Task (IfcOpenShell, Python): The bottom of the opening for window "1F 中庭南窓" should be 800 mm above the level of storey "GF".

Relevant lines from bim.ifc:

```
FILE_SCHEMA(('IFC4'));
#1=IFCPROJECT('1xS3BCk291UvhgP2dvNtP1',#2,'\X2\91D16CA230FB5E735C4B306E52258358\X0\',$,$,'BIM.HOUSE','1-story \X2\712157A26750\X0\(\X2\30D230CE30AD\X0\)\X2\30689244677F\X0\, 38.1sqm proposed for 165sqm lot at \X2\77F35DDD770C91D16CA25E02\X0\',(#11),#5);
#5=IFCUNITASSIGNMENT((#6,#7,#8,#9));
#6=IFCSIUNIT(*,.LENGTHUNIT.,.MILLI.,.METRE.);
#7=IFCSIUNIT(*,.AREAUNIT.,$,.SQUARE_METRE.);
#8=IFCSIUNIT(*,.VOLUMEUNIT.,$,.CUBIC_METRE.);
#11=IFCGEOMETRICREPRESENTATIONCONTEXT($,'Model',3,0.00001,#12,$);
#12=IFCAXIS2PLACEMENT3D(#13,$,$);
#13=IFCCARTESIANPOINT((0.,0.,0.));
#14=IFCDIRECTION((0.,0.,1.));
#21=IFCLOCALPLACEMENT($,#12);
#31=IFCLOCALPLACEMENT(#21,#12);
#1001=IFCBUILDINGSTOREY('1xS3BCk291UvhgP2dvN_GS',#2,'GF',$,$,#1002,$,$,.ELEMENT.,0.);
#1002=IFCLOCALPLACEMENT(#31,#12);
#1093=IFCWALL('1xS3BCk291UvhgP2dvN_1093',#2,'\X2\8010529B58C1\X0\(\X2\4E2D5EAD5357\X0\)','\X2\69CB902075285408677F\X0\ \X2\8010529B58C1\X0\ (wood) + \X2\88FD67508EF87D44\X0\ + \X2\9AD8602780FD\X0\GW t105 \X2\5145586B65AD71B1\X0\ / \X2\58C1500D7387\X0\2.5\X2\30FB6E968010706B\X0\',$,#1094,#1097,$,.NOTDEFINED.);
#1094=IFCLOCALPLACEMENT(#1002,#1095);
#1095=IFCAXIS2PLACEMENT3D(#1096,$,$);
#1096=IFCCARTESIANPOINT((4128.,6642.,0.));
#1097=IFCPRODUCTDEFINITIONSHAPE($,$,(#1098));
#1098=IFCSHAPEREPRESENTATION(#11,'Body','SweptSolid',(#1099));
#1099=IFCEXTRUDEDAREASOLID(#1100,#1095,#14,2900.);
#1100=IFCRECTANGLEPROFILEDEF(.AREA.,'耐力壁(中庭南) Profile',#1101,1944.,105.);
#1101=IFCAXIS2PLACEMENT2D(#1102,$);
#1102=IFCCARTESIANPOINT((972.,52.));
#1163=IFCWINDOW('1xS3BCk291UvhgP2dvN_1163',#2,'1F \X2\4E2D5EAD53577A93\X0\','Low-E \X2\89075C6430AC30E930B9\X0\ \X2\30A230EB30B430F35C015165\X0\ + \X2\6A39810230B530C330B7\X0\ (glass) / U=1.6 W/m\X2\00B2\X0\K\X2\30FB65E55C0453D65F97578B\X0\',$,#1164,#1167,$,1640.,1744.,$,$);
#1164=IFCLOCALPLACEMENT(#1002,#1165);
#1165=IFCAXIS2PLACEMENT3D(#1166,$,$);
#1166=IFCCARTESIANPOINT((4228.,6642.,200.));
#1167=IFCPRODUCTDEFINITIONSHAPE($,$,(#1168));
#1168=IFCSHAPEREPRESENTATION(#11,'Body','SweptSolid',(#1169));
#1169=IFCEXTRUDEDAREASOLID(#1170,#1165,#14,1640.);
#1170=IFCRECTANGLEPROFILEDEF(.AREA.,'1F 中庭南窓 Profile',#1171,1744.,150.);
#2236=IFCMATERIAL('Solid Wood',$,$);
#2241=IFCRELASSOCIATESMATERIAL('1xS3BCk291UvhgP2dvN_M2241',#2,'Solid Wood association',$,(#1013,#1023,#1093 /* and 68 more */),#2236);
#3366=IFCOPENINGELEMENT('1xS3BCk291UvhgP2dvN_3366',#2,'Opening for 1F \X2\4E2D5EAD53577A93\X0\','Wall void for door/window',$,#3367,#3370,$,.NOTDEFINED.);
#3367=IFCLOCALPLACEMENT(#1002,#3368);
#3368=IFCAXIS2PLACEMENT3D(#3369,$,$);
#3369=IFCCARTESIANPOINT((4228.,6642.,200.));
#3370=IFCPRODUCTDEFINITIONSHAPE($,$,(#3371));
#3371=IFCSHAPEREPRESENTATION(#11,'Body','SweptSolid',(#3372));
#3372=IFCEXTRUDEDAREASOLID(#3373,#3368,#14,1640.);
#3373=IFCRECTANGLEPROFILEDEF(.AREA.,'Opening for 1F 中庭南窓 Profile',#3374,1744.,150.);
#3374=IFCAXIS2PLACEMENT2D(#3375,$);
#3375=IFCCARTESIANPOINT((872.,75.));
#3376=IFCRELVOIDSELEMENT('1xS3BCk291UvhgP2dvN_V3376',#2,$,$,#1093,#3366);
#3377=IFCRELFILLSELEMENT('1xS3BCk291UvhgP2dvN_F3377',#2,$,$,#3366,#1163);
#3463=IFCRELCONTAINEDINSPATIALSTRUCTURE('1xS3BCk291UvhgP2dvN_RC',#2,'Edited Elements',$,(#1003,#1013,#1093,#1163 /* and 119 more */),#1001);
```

```python
import numpy as np
import ifcopenshell
import ifcopenshell.api.geometry
import ifcopenshell.geom
import ifcopenshell.util.element
import ifcopenshell.util.placement
import ifcopenshell.util.shape
import ifcopenshell.util.unit

model = ifcopenshell.open("bim.ifc")
unit_scale = ifcopenshell.util.unit.calculate_unit_scale(model)

window = model.by_guid("1xS3BCk291UvhgP2dvN_1163")
opening = window.FillsVoids[0].RelatingOpeningElement
storey = ifcopenshell.util.element.get_container(window, ifc_class="IfcBuildingStorey")
level = ifcopenshell.util.placement.get_local_placement(storey.ObjectPlacement)[2, 3]

# The opening's origin need not be at the sill, so measure its lowest point.
shape = ifcopenshell.geom.create_shape(ifcopenshell.geom.settings(), opening)
bottom = ifcopenshell.util.shape.get_shape_bottom_elevation(shape, shape.geometry) / unit_scale
dz = level + 0.8 / unit_scale - bottom

shift = np.array([0.0, 0.0, dz])
# The window is not placed relative to its opening, so move both.
for product in (opening, window):
    matrix = ifcopenshell.util.placement.get_local_placement(product.ObjectPlacement)
    matrix[:3, 3] += shift
    ifcopenshell.api.geometry.edit_object_placement(model, product=product, matrix=matrix, is_si=False)

print(f"moved by {dz * unit_scale:+.3f} m")

model.write("bim_edited.ifc")
```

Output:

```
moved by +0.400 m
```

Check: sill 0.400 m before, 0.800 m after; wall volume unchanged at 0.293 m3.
